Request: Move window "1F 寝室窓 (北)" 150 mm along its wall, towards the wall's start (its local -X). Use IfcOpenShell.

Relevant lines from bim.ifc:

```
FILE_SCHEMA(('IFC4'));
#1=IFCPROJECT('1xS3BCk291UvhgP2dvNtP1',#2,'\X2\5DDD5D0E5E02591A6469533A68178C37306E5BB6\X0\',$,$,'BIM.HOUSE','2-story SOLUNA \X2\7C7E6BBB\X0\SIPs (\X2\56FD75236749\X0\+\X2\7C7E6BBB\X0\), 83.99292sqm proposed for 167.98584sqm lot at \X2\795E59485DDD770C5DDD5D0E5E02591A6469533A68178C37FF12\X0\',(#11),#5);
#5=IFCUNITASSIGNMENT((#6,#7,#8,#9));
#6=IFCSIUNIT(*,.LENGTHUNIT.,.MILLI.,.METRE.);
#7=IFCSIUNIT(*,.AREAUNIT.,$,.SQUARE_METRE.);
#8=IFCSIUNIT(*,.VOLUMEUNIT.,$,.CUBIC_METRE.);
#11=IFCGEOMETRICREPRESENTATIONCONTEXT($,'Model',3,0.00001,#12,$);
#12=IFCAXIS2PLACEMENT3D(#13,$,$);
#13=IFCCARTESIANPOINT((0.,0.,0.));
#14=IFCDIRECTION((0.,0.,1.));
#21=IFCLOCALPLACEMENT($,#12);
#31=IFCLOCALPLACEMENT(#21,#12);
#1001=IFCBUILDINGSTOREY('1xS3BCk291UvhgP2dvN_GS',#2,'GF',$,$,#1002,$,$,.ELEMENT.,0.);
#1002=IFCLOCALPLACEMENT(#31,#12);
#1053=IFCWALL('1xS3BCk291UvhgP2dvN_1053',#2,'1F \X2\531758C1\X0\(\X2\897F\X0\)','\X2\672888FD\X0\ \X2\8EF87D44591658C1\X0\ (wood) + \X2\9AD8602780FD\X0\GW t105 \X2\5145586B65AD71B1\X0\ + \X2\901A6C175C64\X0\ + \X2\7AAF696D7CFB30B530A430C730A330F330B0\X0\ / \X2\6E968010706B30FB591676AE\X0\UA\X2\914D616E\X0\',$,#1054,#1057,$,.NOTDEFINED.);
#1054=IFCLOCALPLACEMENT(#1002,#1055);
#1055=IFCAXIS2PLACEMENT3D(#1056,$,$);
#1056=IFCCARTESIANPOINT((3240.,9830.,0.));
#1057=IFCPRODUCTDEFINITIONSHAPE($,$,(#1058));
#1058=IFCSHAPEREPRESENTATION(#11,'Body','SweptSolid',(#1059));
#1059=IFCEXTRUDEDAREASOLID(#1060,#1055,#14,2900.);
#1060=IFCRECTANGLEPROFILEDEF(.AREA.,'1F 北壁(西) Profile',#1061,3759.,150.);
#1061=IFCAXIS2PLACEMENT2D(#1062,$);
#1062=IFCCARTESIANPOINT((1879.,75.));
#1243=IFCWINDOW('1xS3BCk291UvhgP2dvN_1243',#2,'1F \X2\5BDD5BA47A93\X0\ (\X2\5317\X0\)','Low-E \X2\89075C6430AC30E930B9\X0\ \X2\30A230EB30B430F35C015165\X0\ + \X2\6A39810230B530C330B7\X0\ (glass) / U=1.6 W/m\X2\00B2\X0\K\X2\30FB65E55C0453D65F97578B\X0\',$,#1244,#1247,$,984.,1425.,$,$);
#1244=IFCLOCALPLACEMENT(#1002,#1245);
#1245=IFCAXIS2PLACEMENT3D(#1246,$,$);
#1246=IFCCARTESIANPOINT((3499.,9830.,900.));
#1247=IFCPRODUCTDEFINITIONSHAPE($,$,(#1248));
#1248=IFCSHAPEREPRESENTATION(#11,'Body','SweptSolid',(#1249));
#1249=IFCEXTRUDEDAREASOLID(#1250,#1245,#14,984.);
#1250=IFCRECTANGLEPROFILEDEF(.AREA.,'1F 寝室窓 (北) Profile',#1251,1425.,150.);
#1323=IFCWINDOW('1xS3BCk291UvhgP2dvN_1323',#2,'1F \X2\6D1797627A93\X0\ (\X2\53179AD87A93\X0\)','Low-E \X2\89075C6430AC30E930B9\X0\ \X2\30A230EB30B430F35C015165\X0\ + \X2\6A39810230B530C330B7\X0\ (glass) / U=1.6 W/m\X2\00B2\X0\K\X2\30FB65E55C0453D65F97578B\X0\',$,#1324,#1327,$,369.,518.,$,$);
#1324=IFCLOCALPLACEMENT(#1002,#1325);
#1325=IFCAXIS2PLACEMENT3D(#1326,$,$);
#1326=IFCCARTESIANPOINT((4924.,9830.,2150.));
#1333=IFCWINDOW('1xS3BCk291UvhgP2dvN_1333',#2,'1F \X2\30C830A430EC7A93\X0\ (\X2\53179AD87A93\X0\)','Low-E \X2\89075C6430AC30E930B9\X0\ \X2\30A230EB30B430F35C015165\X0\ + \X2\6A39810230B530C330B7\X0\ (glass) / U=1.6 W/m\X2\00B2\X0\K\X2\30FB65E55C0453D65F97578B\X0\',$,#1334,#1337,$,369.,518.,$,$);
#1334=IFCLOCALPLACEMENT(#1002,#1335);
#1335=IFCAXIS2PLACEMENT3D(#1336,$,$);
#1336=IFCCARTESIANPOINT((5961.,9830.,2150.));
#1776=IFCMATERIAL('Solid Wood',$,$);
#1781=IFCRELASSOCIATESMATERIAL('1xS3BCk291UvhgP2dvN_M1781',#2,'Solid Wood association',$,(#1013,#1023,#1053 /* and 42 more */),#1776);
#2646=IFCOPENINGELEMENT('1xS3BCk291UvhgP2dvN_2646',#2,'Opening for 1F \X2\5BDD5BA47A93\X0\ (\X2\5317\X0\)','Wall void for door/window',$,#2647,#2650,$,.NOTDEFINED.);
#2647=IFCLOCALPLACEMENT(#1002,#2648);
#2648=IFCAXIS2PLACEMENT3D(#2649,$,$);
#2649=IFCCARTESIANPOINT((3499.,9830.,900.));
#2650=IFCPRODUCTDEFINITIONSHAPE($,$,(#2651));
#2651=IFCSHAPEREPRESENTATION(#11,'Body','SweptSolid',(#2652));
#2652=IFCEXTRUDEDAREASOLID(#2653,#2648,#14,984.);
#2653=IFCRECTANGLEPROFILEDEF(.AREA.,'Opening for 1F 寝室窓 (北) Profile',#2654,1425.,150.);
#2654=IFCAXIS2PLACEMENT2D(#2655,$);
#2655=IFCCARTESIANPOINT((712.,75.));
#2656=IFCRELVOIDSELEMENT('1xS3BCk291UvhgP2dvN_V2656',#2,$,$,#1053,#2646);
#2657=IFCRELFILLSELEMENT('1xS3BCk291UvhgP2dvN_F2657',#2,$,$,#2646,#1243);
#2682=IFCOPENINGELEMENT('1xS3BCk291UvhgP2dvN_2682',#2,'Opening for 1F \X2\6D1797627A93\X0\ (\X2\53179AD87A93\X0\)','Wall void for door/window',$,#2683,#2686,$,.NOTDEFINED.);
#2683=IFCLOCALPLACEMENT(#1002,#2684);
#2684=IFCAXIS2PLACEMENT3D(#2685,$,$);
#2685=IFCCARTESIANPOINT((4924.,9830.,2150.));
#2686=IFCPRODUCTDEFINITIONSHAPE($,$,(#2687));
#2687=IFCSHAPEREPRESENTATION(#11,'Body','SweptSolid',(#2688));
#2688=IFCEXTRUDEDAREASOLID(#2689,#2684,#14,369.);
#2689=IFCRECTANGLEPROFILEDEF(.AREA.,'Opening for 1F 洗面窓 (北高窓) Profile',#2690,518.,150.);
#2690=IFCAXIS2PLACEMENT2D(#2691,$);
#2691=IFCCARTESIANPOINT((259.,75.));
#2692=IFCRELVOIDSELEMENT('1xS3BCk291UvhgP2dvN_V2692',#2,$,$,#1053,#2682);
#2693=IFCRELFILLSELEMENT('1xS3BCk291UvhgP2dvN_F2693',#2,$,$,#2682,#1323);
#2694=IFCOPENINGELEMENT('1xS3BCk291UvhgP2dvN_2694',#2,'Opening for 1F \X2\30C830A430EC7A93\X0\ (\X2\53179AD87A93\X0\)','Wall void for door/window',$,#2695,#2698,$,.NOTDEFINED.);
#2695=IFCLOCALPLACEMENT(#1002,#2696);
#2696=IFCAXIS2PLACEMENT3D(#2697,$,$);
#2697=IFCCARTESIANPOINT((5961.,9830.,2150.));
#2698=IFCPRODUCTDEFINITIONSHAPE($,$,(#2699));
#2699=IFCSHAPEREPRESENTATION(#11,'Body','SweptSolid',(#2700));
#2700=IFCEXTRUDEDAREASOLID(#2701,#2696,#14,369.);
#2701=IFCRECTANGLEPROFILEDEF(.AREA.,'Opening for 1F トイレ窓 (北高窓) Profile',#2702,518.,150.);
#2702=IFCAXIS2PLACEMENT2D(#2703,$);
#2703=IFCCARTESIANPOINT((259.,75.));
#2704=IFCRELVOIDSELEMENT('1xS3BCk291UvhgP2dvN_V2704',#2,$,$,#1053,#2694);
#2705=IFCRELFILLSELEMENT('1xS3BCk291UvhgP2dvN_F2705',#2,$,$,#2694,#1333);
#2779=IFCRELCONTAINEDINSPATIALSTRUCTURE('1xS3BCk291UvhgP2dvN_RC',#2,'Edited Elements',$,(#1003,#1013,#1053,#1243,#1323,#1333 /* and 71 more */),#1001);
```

```python
import ifcopenshell
import ifcopenshell.api.geometry
import ifcopenshell.util.placement
import ifcopenshell.util.unit

model = ifcopenshell.open("bim.ifc")
unit_scale = ifcopenshell.util.unit.calculate_unit_scale(model)

window = model.by_guid("1xS3BCk291UvhgP2dvN_1243")
opening = window.FillsVoids[0].RelatingOpeningElement
wall = opening.VoidsElements[0].RelatingBuildingElement

wall_matrix = ifcopenshell.util.placement.get_local_placement(wall.ObjectPlacement)
shift = wall_matrix[:3, 0] * -0.15 / unit_scale
before = ifcopenshell.util.placement.get_local_placement(window.ObjectPlacement)[:3, 3].copy()

# The window is not placed relative to its opening, so move both.
for product in (opening, window):
    matrix = ifcopenshell.util.placement.get_local_placement(product.ObjectPlacement)
    matrix[:3, 3] += shift
    ifcopenshell.api.geometry.edit_object_placement(model, product=product, matrix=matrix, is_si=False)

after = ifcopenshell.util.placement.get_local_placement(window.ObjectPlacement)[:3, 3]
print("window moved by", (after - before).round(3) + 0.0)

model.write("bim_updated.ifc")
```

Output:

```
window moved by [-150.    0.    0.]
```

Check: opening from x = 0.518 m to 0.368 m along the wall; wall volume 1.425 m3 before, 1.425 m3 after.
